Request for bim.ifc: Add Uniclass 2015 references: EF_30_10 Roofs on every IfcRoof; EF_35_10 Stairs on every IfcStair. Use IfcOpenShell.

First a look at what the model holds.

```python
import ifcopenshell

model = ifcopenshell.open("bim.ifc")
print(model.schema)
print("classifications:", [c.Name for c in model.by_type("IfcClassification")])
for ifc_class in ("IfcDoor", "IfcRoof", "IfcStair", "IfcWall", "IfcWindow"):
    print(ifc_class, len(model.by_type(ifc_class)))
```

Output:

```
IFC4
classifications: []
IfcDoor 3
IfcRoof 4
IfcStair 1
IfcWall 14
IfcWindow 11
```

```python
import ifcopenshell
import ifcopenshell.api.classification

model = ifcopenshell.open("bim.ifc")

system = ifcopenshell.api.classification.add_classification(model, classification="Uniclass 2015")

codes = {
    "IfcRoof": ("EF_30_10", "Roofs"),
    "IfcStair": ("EF_35_10", "Stairs"),
}
for ifc_class, (code, name) in codes.items():
    products = model.by_type(ifc_class)
    ifcopenshell.api.classification.add_reference(
        model, products=products, classification=system, identification=code, name=name
    )
    print(code, len(products))

model.write("bim_rev.ifc")
```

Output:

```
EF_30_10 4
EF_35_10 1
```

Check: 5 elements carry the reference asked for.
